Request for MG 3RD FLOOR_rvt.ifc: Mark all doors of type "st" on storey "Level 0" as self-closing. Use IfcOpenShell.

First a look at what the model holds.

```python
import ifcopenshell
import ifcopenshell.util.element

model = ifcopenshell.open("MG 3RD FLOOR_rvt.ifc")
print(model.schema)
storey = next(s for s in model.by_type("IfcBuildingStorey") if s.Name == "Level 0")
doors = [e for e in ifcopenshell.util.element.get_decomposition(storey) if e.is_a("IfcDoor")]
seen = {}
for e in doors:
    element_type = ifcopenshell.util.element.get_type(e)
    key = (element_type.Name if element_type != e and element_type else None, ifcopenshell.util.element.get_pset(e, "Pset_DoorCommon", "SelfClosing"))
    seen[key] = seen.get(key, 0) + 1
for (name, value), count in sorted(seen.items(), key=str):
    print(count, "x", name, "|", value)
```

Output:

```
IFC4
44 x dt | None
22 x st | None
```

```python
import ifcopenshell
import ifcopenshell.api.pset
import ifcopenshell.util.element

model = ifcopenshell.open("MG 3RD FLOOR_rvt.ifc")

storey = next(s for s in model.by_type("IfcBuildingStorey") if s.Name == "Level 0")
doors = [e for e in ifcopenshell.util.element.get_decomposition(storey) if e.is_a("IfcDoor")]

count = 0
for e in doors:
    element_type = ifcopenshell.util.element.get_type(e)
    if element_type in (None, e) or element_type.Name != "st":
        continue
    # add_pset returns the element's existing set when there is one.
    pset = ifcopenshell.api.pset.add_pset(model, product=e, name="Pset_DoorCommon")
    ifcopenshell.api.pset.edit_pset(model, pset=pset, properties={"SelfClosing": True})
    count += 1

print(count, "doors updated")

model.write("MG 3RD FLOOR_rvt_edited.ifc")
```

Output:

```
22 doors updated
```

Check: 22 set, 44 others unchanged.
